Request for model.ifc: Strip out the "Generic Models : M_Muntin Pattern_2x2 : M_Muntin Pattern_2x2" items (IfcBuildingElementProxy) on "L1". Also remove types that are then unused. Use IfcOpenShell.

First a look at what the model holds.

```python
import ifcopenshell
import ifcopenshell.util.element

model = ifcopenshell.open("model.ifc")
print(model.schema)
storey = next(s for s in model.by_type("IfcBuildingStorey") if s.Name == "L1")
proxies = [e for e in ifcopenshell.util.element.get_decomposition(storey) if e.is_a("IfcBuildingElementProxy")]
seen = {}
for e in proxies:
    element_type = ifcopenshell.util.element.get_type(e)
    name = element_type.Name if element_type not in (None, e) else None
    seen[name] = seen.get(name, 0) + 1
for name, count in sorted(seen.items(), key=str):
    print(count, "x", name)
```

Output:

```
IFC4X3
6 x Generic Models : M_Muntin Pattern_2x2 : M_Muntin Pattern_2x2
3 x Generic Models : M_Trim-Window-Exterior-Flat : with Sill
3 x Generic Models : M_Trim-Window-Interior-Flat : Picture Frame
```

```python
import ifcopenshell
import ifcopenshell.api.root
import ifcopenshell.util.element

model = ifcopenshell.open("model.ifc")

storey = next(s for s in model.by_type("IfcBuildingStorey") if s.Name == "L1")
proxies = [e for e in ifcopenshell.util.element.get_decomposition(storey) if e.is_a("IfcBuildingElementProxy")]
targets = [e for e in proxies if (t := ifcopenshell.util.element.get_type(e)) not in (None, e) and t.Name == "Generic Models : M_Muntin Pattern_2x2 : M_Muntin Pattern_2x2"]
types = {ifcopenshell.util.element.get_type(e) for e in targets} - {None, *targets}

for e in targets:
    ifcopenshell.api.root.remove_product(model, product=e)
print(len(targets), "removed")

unused = [t for t in types if not ifcopenshell.util.element.get_types(t)]
for t in unused:
    ifcopenshell.api.root.remove_product(model, product=t)
print(len(unused), "unused types removed")

model.write("model-out.ifc")
```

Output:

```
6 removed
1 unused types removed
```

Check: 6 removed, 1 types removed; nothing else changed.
